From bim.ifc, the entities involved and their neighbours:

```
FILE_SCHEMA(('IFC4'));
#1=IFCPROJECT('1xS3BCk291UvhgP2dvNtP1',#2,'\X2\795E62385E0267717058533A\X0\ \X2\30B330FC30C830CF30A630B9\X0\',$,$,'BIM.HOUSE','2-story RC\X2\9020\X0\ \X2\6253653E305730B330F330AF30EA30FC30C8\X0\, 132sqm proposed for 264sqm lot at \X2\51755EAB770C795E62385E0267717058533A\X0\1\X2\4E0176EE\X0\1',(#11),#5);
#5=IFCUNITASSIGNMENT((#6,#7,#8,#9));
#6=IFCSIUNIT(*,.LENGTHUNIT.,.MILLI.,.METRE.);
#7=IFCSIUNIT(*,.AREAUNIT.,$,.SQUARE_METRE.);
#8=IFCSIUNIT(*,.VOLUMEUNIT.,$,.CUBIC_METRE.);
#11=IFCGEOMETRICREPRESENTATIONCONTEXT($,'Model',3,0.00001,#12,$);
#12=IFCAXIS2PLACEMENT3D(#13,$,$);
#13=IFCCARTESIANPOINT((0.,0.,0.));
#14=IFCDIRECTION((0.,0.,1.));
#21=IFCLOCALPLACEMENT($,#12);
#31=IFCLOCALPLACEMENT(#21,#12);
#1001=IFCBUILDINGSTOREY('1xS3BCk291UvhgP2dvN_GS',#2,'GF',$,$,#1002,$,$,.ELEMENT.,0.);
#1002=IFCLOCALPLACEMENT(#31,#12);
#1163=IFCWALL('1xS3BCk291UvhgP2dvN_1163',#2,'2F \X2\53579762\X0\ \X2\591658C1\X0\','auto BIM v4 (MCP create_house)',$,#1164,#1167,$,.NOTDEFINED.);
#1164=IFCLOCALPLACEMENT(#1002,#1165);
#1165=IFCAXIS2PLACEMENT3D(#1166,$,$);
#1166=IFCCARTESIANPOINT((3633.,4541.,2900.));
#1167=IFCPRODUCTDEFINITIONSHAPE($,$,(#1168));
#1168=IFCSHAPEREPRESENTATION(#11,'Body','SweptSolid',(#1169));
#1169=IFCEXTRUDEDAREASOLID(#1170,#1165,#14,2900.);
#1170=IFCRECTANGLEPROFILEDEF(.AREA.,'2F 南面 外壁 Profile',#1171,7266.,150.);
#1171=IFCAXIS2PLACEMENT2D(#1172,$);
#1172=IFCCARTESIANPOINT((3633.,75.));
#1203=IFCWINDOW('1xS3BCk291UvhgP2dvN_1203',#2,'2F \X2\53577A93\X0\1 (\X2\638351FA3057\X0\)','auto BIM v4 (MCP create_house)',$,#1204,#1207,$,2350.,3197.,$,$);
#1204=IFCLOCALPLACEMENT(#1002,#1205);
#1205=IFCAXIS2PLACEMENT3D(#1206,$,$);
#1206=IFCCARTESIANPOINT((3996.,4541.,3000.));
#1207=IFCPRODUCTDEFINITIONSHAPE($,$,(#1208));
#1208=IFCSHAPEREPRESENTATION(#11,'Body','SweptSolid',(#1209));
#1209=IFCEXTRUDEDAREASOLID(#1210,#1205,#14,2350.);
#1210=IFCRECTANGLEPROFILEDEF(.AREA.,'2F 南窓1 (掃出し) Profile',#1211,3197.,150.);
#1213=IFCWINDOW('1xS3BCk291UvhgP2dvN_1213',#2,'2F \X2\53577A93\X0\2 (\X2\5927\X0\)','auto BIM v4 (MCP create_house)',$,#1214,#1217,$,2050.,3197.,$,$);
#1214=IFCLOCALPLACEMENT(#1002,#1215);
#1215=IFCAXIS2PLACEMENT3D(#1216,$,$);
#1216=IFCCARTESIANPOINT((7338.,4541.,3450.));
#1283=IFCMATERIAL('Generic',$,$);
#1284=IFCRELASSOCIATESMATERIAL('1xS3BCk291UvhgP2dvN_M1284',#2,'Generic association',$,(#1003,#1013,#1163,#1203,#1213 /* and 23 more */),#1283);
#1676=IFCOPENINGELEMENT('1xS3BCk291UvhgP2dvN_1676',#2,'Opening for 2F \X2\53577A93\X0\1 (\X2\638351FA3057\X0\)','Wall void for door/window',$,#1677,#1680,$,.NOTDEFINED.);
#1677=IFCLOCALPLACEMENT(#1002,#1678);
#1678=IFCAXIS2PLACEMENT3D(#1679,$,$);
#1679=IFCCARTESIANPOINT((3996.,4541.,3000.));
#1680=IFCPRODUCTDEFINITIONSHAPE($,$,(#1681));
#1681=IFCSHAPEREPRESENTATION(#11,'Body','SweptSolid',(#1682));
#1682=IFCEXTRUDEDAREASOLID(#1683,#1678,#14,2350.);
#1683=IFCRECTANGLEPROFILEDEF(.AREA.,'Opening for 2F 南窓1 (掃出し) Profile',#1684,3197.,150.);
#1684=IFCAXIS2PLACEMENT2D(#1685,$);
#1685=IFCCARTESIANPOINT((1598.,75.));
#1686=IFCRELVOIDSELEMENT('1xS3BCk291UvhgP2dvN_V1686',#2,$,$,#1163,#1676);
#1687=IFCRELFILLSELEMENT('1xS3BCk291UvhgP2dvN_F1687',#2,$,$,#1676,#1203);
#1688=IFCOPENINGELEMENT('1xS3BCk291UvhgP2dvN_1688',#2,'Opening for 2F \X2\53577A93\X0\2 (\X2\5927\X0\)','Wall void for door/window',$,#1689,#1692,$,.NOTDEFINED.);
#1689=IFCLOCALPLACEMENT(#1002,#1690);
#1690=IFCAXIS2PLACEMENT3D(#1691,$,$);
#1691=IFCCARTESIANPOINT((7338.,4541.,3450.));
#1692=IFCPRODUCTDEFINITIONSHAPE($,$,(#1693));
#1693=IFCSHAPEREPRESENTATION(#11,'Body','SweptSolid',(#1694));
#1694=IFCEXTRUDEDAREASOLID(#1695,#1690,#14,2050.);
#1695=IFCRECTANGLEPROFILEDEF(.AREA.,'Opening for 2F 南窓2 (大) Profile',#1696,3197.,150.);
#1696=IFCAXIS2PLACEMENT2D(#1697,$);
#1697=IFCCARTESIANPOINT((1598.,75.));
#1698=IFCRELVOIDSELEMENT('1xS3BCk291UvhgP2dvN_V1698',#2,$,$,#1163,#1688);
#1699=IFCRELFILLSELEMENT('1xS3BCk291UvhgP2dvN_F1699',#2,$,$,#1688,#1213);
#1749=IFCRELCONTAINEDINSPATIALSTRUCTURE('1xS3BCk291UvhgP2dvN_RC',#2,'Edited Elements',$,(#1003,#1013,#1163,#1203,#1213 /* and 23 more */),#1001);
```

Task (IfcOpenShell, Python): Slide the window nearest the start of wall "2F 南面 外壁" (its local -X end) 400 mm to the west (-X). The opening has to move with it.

```python
import ifcopenshell
import ifcopenshell.api.geometry
import ifcopenshell.util.placement
import ifcopenshell.util.unit

model = ifcopenshell.open("bim.ifc")
unit_scale = ifcopenshell.util.unit.calculate_unit_scale(model)

window = model.by_id(1203)
opening = window.FillsVoids[0].RelatingOpeningElement
wall = opening.VoidsElements[0].RelatingBuildingElement

wall_matrix = ifcopenshell.util.placement.get_local_placement(wall.ObjectPlacement)
shift = wall_matrix[:3, 0] * -0.4 / unit_scale
before = ifcopenshell.util.placement.get_local_placement(window.ObjectPlacement)[:3, 3].copy()

# The window is not placed relative to its opening, so move both.
for product in (opening, window):
    matrix = ifcopenshell.util.placement.get_local_placement(product.ObjectPlacement)
    matrix[:3, 3] += shift
    ifcopenshell.api.geometry.edit_object_placement(model, product=product, matrix=matrix, is_si=False)

after = ifcopenshell.util.placement.get_local_placement(window.ObjectPlacement)[:3, 3]
print("window moved by", (after - before).round(3) + 0.0)

model.write("bim_updated.ifc")
```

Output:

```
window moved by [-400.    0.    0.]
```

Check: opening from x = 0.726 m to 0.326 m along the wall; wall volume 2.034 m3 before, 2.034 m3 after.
